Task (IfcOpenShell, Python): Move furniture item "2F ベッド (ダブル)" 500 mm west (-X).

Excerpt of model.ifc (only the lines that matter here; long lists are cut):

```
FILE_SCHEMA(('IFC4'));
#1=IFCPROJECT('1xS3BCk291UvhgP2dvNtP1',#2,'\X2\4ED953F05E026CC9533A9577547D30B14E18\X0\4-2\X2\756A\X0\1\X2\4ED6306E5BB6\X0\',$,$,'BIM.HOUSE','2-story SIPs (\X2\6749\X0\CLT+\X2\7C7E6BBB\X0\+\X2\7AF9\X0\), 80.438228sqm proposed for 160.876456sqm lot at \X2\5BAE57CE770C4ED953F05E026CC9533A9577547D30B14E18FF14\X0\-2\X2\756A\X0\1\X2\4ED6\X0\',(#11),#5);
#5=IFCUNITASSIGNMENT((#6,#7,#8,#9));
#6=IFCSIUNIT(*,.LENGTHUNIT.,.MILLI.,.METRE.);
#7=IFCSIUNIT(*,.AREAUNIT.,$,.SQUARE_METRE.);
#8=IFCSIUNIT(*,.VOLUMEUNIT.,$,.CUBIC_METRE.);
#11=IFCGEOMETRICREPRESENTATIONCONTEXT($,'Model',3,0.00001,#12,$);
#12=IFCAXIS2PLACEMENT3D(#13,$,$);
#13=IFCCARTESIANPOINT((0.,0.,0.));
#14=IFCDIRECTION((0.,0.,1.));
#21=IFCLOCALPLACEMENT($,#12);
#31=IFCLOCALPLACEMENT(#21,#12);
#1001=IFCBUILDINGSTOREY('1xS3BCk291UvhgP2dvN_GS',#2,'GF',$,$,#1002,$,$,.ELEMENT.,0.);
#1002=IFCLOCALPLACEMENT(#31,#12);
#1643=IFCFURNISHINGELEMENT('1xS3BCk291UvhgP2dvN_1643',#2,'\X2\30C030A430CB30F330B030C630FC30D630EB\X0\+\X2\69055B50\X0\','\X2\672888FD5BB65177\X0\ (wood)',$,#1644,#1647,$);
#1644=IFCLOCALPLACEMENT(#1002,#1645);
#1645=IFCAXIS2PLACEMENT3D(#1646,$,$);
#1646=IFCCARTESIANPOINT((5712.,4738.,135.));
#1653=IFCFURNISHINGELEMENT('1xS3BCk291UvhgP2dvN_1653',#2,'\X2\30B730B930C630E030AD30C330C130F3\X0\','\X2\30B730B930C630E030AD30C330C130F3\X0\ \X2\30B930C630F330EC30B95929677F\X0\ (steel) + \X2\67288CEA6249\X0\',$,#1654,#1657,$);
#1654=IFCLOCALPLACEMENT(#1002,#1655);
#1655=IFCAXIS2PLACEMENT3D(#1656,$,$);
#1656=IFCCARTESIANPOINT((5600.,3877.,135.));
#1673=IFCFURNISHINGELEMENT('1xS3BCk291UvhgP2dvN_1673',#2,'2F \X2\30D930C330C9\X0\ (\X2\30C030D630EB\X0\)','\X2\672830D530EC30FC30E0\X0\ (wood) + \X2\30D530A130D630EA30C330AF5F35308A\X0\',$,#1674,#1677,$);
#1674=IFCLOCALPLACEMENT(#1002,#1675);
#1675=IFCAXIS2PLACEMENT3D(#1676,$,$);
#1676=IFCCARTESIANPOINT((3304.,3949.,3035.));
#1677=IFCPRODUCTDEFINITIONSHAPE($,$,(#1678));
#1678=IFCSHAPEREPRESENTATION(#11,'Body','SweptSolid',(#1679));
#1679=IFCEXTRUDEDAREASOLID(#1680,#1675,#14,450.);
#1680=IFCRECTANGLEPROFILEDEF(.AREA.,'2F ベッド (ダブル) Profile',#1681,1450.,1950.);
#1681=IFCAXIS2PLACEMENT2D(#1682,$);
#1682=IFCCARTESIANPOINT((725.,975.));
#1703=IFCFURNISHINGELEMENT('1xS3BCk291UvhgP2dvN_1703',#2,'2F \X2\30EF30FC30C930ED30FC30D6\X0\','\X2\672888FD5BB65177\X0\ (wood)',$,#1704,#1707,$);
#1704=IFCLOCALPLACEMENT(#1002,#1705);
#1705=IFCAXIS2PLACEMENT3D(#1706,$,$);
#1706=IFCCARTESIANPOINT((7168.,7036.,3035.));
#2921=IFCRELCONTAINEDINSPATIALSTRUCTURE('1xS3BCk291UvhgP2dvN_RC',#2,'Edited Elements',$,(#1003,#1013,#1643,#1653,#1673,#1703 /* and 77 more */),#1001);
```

```python
import ifcopenshell
import ifcopenshell.api.geometry
import ifcopenshell.util.placement

model = ifcopenshell.open("model.ifc")

item = model.by_guid("1xS3BCk291UvhgP2dvN_1673")
matrix = ifcopenshell.util.placement.get_local_placement(item.ObjectPlacement)
matrix[0, 3] -= 500.0
ifcopenshell.api.geometry.edit_object_placement(model, product=item, matrix=matrix, is_si=False)

print(ifcopenshell.util.placement.get_local_placement(item.ObjectPlacement).round(3) + 0.0)

model.write("model_v2.ifc")
```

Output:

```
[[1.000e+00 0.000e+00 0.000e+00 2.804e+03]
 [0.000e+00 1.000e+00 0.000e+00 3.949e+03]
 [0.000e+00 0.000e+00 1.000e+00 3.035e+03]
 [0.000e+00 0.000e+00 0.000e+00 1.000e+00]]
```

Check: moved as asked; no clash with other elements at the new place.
